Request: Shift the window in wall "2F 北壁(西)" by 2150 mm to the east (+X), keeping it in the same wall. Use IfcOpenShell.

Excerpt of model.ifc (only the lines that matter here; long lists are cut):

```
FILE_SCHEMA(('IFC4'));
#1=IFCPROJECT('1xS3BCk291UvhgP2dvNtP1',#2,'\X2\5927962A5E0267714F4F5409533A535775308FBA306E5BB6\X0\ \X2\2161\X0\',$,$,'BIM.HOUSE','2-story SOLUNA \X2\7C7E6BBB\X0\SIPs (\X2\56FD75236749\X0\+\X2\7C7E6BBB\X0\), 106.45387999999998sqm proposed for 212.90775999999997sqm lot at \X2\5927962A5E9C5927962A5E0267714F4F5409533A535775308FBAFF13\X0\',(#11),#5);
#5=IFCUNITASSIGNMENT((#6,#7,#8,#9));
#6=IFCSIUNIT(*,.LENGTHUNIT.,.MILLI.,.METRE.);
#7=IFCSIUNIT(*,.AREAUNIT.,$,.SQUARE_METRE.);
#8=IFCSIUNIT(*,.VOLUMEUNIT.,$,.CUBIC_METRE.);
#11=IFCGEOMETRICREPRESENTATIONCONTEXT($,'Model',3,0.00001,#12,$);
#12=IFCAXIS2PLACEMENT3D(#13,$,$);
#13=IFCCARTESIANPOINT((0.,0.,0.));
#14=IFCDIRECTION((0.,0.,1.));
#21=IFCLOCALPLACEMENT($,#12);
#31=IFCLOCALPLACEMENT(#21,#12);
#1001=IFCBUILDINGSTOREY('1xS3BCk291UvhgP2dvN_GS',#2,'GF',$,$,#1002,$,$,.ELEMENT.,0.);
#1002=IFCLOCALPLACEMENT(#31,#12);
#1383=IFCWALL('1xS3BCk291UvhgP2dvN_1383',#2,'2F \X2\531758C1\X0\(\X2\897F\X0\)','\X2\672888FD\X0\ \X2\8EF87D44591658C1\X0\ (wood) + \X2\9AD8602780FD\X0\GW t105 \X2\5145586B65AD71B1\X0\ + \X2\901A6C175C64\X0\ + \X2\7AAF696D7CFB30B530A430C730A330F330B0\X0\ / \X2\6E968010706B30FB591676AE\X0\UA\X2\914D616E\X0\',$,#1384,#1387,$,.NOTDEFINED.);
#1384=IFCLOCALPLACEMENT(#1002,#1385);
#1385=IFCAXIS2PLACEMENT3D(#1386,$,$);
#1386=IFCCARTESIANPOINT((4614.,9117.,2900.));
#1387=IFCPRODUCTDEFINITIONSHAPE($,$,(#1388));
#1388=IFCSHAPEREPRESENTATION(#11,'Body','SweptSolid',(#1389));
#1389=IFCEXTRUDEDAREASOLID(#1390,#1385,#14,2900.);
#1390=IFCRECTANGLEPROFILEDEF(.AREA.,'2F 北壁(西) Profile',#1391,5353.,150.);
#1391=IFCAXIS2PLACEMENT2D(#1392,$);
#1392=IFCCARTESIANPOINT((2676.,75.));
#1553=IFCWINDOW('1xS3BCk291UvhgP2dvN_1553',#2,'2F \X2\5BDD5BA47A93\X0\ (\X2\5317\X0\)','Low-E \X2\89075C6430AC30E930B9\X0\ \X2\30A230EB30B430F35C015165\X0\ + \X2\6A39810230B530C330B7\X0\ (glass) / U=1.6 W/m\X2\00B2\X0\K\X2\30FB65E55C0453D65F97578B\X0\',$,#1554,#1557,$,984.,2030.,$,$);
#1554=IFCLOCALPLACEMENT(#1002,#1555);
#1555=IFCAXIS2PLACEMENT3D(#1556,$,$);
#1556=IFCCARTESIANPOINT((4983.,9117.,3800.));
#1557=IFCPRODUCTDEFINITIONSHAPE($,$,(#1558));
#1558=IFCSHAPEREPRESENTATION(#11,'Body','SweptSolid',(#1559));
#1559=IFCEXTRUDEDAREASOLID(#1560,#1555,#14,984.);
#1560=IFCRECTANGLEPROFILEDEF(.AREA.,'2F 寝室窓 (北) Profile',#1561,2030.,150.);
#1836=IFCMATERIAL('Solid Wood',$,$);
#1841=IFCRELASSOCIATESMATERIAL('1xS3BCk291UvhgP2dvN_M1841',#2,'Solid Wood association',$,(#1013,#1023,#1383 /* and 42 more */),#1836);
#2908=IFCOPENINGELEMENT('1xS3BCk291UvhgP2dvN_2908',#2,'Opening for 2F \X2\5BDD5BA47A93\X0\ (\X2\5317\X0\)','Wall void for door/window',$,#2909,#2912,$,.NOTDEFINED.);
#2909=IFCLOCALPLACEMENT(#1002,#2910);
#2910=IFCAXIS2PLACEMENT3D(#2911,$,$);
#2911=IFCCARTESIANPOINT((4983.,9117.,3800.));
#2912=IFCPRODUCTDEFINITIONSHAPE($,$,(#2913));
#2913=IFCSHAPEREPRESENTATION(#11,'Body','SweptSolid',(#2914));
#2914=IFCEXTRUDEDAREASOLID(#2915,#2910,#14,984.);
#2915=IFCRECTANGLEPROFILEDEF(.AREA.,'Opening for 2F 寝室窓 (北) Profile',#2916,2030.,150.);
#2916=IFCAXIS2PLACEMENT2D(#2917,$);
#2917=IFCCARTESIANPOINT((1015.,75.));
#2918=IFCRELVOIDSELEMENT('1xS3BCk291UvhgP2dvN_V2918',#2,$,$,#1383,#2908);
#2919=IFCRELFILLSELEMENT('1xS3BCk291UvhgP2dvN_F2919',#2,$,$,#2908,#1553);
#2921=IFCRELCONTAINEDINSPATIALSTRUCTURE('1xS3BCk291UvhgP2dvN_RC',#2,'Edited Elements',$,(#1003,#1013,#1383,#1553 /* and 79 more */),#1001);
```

```python
import ifcopenshell
import ifcopenshell.api.geometry
import ifcopenshell.util.placement
import ifcopenshell.util.unit

model = ifcopenshell.open("model.ifc")
unit_scale = ifcopenshell.util.unit.calculate_unit_scale(model)

window = model.by_guid("1xS3BCk291UvhgP2dvN_1553")
opening = window.FillsVoids[0].RelatingOpeningElement
wall = opening.VoidsElements[0].RelatingBuildingElement

wall_matrix = ifcopenshell.util.placement.get_local_placement(wall.ObjectPlacement)
shift = wall_matrix[:3, 0] * 2.15 / unit_scale
before = ifcopenshell.util.placement.get_local_placement(window.ObjectPlacement)[:3, 3].copy()

# The window is not placed relative to its opening, so move both.
for product in (opening, window):
    matrix = ifcopenshell.util.placement.get_local_placement(product.ObjectPlacement)
    matrix[:3, 3] += shift
    ifcopenshell.api.geometry.edit_object_placement(model, product=product, matrix=matrix, is_si=False)

after = ifcopenshell.util.placement.get_local_placement(window.ObjectPlacement)[:3, 3]
print("window moved by", (after - before).round(3) + 0.0)

model.write("model_edited.ifc")
```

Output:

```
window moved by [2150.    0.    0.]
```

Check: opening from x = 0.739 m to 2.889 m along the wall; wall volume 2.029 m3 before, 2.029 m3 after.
